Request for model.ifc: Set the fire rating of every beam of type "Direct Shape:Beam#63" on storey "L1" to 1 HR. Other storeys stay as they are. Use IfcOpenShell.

First a look at what the model holds.

```python
import ifcopenshell
import ifcopenshell.util.element

model = ifcopenshell.open("model.ifc")
print(model.schema)
storey = next(s for s in model.by_type("IfcBuildingStorey") if s.Name == "L1")
beams = [e for e in ifcopenshell.util.element.get_decomposition(storey) if e.is_a("IfcBeam")]
seen = {}
for e in beams:
    element_type = ifcopenshell.util.element.get_type(e)
    key = (element_type.Name if element_type != e and element_type else None, ifcopenshell.util.element.get_pset(e, "Pset_BeamCommon", "FireRating"))
    seen[key] = seen.get(key, 0) + 1
for (name, value), count in sorted(seen.items(), key=str):
    print(count, "x", name, "|", value)
```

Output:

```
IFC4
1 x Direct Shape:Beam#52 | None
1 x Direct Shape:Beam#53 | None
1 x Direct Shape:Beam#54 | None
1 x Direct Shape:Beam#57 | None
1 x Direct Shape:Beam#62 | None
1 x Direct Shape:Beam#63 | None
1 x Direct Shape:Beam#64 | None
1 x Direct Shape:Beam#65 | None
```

```python
import ifcopenshell
import ifcopenshell.api.pset
import ifcopenshell.util.element

model = ifcopenshell.open("model.ifc")

storey = next(s for s in model.by_type("IfcBuildingStorey") if s.Name == "L1")
beams = [e for e in ifcopenshell.util.element.get_decomposition(storey) if e.is_a("IfcBeam")]

count = 0
for e in beams:
    element_type = ifcopenshell.util.element.get_type(e)
    if element_type in (None, e) or element_type.Name != "Direct Shape:Beam#63":
        continue
    # add_pset returns the element's existing set when there is one.
    pset = ifcopenshell.api.pset.add_pset(model, product=e, name="Pset_BeamCommon")
    ifcopenshell.api.pset.edit_pset(model, pset=pset, properties={"FireRating": "1 HR"})
    count += 1

print(count, "beams updated")

model.write("model-out.ifc")
```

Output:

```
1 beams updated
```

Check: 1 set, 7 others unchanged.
